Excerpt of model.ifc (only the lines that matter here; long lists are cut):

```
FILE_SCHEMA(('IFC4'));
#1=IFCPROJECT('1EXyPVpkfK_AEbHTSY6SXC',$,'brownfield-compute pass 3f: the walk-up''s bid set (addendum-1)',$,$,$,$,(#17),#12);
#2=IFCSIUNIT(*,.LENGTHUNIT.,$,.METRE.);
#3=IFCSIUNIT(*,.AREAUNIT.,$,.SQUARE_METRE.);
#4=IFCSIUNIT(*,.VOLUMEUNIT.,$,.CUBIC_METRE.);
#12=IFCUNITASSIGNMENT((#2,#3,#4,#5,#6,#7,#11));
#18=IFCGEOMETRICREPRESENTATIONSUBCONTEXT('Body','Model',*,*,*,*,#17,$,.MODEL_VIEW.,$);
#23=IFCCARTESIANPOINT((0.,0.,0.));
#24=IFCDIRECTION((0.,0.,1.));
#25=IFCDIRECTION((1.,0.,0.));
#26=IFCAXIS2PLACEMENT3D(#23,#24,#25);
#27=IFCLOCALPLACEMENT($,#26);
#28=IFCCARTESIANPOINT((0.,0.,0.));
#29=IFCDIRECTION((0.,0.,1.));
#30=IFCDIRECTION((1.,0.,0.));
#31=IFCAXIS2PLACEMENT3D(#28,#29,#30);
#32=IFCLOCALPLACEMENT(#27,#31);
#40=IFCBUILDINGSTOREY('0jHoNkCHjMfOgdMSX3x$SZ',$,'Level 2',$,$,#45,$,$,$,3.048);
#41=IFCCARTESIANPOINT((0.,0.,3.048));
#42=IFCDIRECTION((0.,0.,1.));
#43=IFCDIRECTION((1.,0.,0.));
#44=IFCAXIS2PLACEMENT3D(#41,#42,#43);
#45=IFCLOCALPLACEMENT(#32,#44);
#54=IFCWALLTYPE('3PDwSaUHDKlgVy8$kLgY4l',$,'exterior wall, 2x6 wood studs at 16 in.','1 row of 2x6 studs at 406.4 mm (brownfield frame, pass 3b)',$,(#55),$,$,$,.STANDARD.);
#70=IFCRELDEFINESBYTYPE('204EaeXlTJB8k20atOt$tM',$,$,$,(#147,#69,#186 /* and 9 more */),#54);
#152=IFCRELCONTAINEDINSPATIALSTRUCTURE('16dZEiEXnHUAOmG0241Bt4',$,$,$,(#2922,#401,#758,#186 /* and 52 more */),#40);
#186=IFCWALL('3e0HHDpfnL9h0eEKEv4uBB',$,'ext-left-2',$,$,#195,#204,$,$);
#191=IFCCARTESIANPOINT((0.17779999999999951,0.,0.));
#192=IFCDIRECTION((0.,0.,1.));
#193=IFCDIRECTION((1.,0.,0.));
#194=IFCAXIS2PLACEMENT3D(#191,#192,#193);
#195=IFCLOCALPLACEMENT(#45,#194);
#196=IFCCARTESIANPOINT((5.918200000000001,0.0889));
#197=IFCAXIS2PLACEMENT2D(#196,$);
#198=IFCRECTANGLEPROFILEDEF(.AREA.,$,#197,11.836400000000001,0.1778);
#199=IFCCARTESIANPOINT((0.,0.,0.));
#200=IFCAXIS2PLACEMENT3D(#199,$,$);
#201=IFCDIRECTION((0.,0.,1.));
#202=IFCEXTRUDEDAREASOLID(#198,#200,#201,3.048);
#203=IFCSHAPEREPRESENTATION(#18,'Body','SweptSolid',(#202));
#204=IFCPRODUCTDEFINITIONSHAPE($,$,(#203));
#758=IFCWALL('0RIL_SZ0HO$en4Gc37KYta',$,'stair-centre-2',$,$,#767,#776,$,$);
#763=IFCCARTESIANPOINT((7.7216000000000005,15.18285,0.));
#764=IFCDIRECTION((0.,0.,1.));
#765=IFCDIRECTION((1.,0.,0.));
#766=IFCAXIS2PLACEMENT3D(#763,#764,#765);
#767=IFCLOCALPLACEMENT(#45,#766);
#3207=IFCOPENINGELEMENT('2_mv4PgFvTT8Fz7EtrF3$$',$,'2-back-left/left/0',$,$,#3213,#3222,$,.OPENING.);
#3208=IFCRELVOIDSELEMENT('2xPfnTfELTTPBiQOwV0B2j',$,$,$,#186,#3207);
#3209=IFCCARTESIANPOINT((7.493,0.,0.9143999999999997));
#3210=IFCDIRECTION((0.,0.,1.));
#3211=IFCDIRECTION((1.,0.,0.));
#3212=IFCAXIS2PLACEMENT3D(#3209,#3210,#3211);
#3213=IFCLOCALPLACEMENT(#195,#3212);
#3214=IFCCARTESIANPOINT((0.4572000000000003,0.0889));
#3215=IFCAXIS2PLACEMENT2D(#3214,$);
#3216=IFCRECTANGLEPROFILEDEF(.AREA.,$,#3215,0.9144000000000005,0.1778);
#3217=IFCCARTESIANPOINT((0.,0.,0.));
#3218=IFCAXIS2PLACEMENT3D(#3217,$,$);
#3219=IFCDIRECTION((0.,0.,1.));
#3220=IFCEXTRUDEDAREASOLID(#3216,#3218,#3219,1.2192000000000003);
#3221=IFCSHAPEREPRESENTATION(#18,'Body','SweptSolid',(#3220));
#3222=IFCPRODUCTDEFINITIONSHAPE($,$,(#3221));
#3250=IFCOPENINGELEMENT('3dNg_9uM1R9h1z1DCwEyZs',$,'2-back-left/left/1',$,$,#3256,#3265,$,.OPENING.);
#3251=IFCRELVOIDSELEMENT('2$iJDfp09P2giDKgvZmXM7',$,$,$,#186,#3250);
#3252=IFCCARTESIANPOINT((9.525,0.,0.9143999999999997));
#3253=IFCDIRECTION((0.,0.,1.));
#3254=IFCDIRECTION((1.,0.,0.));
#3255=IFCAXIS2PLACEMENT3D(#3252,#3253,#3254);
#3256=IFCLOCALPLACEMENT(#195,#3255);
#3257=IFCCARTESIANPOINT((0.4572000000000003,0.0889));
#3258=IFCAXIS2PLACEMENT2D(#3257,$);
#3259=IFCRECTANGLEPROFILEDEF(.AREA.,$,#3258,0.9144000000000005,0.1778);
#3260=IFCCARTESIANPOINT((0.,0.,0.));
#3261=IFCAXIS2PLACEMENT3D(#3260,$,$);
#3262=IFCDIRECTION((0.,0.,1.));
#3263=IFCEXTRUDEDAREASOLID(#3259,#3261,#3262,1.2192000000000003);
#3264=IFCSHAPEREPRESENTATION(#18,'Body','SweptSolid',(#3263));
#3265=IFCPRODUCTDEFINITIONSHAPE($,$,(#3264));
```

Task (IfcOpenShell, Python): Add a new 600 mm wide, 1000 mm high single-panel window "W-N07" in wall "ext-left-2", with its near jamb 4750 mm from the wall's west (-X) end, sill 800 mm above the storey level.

```python
import numpy as np
import ifcopenshell
import ifcopenshell.api.feature
import ifcopenshell.api.geometry
import ifcopenshell.api.root
import ifcopenshell.api.spatial
import ifcopenshell.geom
import ifcopenshell.util.element
import ifcopenshell.util.placement
import ifcopenshell.util.representation
import ifcopenshell.util.shape
import ifcopenshell.util.unit

model = ifcopenshell.open("model.ifc")
unit_scale = ifcopenshell.util.unit.calculate_unit_scale(model)
settings = ifcopenshell.geom.settings()


def volume(element):
    """Net volume in cubic metres, openings subtracted."""
    shape = ifcopenshell.geom.create_shape(settings, element)
    return ifcopenshell.util.shape.get_volume(shape.geometry)


wall = model.by_id(186)
storey = ifcopenshell.util.element.get_container(wall, ifc_class="IfcBuildingStorey")
context = ifcopenshell.util.representation.get_context(model, "Model", "Body", "MODEL_VIEW")
before = volume(wall)

width, height, from_end, sill = 0.6, 1, 4.75, 0.8  # metres

# The wall runs along its own X axis, and the end named is its -X end.
wall_shape = ifcopenshell.geom.create_shape(settings, wall)
x, y, z = ifcopenshell.util.shape.get_vertices(wall_shape.geometry).T
start = x.min() + from_end
face, thickness = float(y.min()), float(y.max() - y.min())
wall_matrix = ifcopenshell.util.placement.get_local_placement(wall.ObjectPlacement)
level = ifcopenshell.util.placement.get_local_placement(storey.ObjectPlacement)[2, 3]


def in_wall(x, y):
    """Placement at x, y metres in the wall's axes, at sill height."""
    matrix = wall_matrix.copy()
    matrix[:, 3] = wall_matrix @ np.array([x / unit_scale, y / unit_scale, 0.0, 1.0])
    matrix[2, 3] = level + sill / unit_scale
    return matrix


# Opening: a box that overshoots both wall faces by 50 mm.
opening = ifcopenshell.api.root.create_entity(model, ifc_class="IfcOpeningElement", predefined_type="OPENING")
box = ifcopenshell.api.geometry.add_wall_representation(
    model, context=context, length=width, height=height, thickness=thickness + 0.1
)
ifcopenshell.api.geometry.assign_representation(model, product=opening, representation=box)
ifcopenshell.api.geometry.edit_object_placement(model, product=opening, matrix=in_wall(start, face - 0.05), is_si=False)
ifcopenshell.api.feature.add_feature(model, feature=opening, element=wall)

window = ifcopenshell.api.root.create_entity(model, ifc_class="IfcWindow", name="W-N07", predefined_type="WINDOW")
window.OverallWidth, window.OverallHeight = width / unit_scale, height / unit_scale
window.PartitioningType = "SINGLE_PANEL"
body = ifcopenshell.api.geometry.add_window_representation(
    model,
    context=context,
    overall_width=window.OverallWidth,
    overall_height=window.OverallHeight,
    partition_type="SINGLE_PANEL",
)
ifcopenshell.api.geometry.assign_representation(model, product=window, representation=body)
ifcopenshell.api.spatial.assign_container(model, products=[window], relating_structure=storey)
ifcopenshell.api.feature.add_filling(model, opening=opening, element=window)

# Centre the window in the wall's thickness.
ifcopenshell.api.geometry.edit_object_placement(model, product=window, matrix=in_wall(start, face), is_si=False)
window_shape = ifcopenshell.geom.create_shape(settings, window)
depth = ifcopenshell.util.shape.get_vertices(window_shape.geometry)[:, 1]
offset = face + thickness / 2 - (depth.min() + depth.max()) / 2
ifcopenshell.api.geometry.edit_object_placement(model, product=window, matrix=in_wall(start, offset), is_si=False)

after = volume(wall)

print(f"wall volume {before:.3f} -> {after:.3f} m3")

model.write("model_rev.ifc")
```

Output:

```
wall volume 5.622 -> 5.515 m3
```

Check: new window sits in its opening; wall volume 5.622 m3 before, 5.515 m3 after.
